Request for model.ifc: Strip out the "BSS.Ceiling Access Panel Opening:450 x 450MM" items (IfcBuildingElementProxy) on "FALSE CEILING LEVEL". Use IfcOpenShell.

First a look at what the model holds.

```python
import ifcopenshell
import ifcopenshell.util.element

model = ifcopenshell.open("model.ifc")
print(model.schema)
storey = next(s for s in model.by_type("IfcBuildingStorey") if s.Name == "FALSE CEILING LEVEL")
proxies = [e for e in ifcopenshell.util.element.get_decomposition(storey) if e.is_a("IfcBuildingElementProxy")]
seen = {}
for e in proxies:
    element_type = ifcopenshell.util.element.get_type(e)
    name = element_type.Name if element_type not in (None, e) else None
    seen[name] = seen.get(name, 0) + 1
for name, count in sorted(seen.items(), key=str):
    print(count, "x", name)
```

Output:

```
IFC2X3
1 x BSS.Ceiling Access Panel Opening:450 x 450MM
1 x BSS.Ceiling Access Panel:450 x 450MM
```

```python
import ifcopenshell
import ifcopenshell.api.root
import ifcopenshell.util.element

model = ifcopenshell.open("model.ifc")

storey = next(s for s in model.by_type("IfcBuildingStorey") if s.Name == "FALSE CEILING LEVEL")
proxies = [e for e in ifcopenshell.util.element.get_decomposition(storey) if e.is_a("IfcBuildingElementProxy")]
targets = [e for e in proxies if (t := ifcopenshell.util.element.get_type(e)) not in (None, e) and t.Name == "BSS.Ceiling Access Panel Opening:450 x 450MM"]

for e in targets:
    ifcopenshell.api.root.remove_product(model, product=e)
print(len(targets), "removed")

model.write("model_edited.ifc")
```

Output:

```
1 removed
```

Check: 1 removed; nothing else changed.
